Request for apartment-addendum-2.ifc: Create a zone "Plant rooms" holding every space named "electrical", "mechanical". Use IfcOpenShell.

First a look at what the model holds.

```python
import ifcopenshell

model = ifcopenshell.open("apartment-addendum-2.ifc")
print(model.schema)
seen = {}
for space in model.by_type("IfcSpace"):
    seen[space.LongName] = seen.get(space.LongName, 0) + 1
for name, count in sorted(seen.items(), key=str):
    print(count, "x", name)
print("zones:", [z.Name for z in model.by_type("IfcZone")][:20])
```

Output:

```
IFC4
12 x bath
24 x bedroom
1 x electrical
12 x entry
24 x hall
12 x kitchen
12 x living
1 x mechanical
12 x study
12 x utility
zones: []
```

```python
import ifcopenshell
import ifcopenshell.api.group
import ifcopenshell.api.root

model = ifcopenshell.open("apartment-addendum-2.ifc")

names = {"electrical", "mechanical"}
spaces = [s for s in model.by_type("IfcSpace") if s.LongName in names]

zone = ifcopenshell.api.root.create_entity(model, ifc_class="IfcZone", name="Plant rooms")
ifcopenshell.api.group.assign_group(model, products=spaces, group=zone)
print(len(spaces), "spaces in", zone.Name)

model.write("apartment-addendum-2_edited.ifc")
```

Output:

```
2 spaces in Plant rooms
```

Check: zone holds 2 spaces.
